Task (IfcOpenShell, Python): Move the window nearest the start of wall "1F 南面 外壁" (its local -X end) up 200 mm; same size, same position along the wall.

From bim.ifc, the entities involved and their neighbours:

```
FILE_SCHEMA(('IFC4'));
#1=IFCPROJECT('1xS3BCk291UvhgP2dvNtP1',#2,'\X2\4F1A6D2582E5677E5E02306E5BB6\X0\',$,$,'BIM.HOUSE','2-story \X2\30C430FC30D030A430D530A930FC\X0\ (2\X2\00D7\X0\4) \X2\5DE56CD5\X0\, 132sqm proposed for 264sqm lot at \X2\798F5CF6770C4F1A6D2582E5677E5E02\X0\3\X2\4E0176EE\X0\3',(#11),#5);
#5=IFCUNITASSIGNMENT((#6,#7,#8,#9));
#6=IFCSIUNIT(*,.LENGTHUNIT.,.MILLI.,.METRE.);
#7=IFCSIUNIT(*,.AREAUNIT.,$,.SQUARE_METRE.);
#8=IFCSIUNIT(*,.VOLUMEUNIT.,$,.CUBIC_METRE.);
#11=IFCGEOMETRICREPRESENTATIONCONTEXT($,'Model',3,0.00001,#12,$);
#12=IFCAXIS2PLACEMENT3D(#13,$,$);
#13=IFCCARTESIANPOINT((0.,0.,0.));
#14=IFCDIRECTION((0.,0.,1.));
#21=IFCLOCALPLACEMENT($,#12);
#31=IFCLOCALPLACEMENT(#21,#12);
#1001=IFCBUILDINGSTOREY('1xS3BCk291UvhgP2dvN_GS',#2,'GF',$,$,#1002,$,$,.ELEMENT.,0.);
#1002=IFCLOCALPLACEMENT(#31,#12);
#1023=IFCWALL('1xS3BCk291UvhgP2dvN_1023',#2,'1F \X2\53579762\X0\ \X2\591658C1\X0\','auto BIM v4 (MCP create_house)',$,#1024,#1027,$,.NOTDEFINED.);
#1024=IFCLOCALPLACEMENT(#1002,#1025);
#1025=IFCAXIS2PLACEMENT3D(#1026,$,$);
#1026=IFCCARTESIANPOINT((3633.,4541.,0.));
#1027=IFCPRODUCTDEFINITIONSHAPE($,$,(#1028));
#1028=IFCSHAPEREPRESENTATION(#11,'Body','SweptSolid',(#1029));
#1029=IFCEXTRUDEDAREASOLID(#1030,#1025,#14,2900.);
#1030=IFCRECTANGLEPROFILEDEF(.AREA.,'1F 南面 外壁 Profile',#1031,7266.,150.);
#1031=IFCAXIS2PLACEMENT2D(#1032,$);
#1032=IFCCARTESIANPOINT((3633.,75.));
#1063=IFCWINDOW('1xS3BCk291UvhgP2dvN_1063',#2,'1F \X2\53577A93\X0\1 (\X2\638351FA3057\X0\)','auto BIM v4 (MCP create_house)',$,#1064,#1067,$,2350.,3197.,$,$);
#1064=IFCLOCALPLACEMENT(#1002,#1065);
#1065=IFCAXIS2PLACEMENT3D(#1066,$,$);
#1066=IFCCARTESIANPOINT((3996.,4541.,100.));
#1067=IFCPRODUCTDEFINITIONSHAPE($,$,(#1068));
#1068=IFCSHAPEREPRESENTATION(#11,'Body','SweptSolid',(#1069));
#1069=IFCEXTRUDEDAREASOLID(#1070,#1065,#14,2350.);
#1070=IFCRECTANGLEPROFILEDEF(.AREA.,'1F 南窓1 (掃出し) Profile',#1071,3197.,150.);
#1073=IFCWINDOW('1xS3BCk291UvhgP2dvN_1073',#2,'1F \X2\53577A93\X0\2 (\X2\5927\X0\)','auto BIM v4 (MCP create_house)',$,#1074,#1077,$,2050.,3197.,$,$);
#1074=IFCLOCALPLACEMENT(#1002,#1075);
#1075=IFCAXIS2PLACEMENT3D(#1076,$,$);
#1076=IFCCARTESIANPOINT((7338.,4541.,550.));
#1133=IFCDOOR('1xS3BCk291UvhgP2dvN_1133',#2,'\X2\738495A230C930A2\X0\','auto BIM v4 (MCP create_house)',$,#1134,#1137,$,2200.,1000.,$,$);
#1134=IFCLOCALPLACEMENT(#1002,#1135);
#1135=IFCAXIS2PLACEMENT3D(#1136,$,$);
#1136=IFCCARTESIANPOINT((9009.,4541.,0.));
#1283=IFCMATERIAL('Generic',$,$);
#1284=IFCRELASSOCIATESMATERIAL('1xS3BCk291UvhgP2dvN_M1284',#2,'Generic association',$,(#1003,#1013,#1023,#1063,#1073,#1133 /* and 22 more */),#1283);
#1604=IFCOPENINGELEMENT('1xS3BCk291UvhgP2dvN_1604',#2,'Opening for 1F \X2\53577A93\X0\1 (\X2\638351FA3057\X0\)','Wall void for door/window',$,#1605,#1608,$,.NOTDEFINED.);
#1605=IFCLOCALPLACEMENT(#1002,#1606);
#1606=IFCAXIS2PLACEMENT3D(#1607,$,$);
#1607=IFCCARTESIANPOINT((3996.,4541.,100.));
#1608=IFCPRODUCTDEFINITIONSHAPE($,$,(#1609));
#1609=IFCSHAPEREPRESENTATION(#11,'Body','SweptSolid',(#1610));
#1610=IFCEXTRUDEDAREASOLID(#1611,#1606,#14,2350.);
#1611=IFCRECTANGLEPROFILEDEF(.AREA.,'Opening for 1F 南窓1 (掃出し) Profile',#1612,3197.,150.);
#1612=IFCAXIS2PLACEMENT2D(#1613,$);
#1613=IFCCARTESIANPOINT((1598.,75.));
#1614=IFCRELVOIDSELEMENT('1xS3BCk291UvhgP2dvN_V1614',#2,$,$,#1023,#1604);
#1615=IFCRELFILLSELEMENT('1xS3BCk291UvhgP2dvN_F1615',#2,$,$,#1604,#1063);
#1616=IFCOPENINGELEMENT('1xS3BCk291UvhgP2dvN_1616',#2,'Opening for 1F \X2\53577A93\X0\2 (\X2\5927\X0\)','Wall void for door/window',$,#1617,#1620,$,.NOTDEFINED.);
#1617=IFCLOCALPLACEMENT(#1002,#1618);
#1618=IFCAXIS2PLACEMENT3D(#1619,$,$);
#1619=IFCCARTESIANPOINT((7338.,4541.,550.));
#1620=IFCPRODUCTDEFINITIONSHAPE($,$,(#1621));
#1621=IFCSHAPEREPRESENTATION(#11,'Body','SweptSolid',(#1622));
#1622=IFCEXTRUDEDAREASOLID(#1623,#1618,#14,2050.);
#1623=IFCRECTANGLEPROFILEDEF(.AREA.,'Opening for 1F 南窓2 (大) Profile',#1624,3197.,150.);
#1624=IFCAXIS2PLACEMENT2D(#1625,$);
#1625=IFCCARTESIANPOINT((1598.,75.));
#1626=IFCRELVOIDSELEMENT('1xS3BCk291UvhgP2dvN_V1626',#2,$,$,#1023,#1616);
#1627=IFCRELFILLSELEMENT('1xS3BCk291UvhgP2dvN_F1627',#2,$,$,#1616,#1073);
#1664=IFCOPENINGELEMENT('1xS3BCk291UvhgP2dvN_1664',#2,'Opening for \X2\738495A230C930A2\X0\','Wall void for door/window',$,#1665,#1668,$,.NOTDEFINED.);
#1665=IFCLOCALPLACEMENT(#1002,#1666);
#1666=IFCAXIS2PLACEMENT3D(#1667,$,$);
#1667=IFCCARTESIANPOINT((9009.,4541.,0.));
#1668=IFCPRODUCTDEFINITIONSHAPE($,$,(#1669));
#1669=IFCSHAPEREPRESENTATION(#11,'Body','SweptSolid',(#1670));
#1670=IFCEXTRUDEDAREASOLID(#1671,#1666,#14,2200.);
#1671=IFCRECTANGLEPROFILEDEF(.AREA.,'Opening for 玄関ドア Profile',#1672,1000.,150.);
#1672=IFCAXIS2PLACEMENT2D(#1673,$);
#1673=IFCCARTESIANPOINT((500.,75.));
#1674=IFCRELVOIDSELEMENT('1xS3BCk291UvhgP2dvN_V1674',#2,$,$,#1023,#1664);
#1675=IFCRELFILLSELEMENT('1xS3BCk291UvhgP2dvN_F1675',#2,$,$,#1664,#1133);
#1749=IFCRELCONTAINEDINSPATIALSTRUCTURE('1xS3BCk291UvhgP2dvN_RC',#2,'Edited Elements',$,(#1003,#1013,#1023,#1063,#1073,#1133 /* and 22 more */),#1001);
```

```python
import numpy as np
import ifcopenshell
import ifcopenshell.api.geometry
import ifcopenshell.util.placement
import ifcopenshell.util.unit

model = ifcopenshell.open("bim.ifc")
unit_scale = ifcopenshell.util.unit.calculate_unit_scale(model)

window = model.by_guid("1xS3BCk291UvhgP2dvN_1063")
opening = window.FillsVoids[0].RelatingOpeningElement
dz = 0.2 / unit_scale

shift = np.array([0.0, 0.0, dz])
# The window is not placed relative to its opening, so move both.
for product in (opening, window):
    matrix = ifcopenshell.util.placement.get_local_placement(product.ObjectPlacement)
    matrix[:3, 3] += shift
    ifcopenshell.api.geometry.edit_object_placement(model, product=product, matrix=matrix, is_si=False)

print(f"moved by {dz * unit_scale:+.3f} m")

model.write("bim_rev.ifc")
```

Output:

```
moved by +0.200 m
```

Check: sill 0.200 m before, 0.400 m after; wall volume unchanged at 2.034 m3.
